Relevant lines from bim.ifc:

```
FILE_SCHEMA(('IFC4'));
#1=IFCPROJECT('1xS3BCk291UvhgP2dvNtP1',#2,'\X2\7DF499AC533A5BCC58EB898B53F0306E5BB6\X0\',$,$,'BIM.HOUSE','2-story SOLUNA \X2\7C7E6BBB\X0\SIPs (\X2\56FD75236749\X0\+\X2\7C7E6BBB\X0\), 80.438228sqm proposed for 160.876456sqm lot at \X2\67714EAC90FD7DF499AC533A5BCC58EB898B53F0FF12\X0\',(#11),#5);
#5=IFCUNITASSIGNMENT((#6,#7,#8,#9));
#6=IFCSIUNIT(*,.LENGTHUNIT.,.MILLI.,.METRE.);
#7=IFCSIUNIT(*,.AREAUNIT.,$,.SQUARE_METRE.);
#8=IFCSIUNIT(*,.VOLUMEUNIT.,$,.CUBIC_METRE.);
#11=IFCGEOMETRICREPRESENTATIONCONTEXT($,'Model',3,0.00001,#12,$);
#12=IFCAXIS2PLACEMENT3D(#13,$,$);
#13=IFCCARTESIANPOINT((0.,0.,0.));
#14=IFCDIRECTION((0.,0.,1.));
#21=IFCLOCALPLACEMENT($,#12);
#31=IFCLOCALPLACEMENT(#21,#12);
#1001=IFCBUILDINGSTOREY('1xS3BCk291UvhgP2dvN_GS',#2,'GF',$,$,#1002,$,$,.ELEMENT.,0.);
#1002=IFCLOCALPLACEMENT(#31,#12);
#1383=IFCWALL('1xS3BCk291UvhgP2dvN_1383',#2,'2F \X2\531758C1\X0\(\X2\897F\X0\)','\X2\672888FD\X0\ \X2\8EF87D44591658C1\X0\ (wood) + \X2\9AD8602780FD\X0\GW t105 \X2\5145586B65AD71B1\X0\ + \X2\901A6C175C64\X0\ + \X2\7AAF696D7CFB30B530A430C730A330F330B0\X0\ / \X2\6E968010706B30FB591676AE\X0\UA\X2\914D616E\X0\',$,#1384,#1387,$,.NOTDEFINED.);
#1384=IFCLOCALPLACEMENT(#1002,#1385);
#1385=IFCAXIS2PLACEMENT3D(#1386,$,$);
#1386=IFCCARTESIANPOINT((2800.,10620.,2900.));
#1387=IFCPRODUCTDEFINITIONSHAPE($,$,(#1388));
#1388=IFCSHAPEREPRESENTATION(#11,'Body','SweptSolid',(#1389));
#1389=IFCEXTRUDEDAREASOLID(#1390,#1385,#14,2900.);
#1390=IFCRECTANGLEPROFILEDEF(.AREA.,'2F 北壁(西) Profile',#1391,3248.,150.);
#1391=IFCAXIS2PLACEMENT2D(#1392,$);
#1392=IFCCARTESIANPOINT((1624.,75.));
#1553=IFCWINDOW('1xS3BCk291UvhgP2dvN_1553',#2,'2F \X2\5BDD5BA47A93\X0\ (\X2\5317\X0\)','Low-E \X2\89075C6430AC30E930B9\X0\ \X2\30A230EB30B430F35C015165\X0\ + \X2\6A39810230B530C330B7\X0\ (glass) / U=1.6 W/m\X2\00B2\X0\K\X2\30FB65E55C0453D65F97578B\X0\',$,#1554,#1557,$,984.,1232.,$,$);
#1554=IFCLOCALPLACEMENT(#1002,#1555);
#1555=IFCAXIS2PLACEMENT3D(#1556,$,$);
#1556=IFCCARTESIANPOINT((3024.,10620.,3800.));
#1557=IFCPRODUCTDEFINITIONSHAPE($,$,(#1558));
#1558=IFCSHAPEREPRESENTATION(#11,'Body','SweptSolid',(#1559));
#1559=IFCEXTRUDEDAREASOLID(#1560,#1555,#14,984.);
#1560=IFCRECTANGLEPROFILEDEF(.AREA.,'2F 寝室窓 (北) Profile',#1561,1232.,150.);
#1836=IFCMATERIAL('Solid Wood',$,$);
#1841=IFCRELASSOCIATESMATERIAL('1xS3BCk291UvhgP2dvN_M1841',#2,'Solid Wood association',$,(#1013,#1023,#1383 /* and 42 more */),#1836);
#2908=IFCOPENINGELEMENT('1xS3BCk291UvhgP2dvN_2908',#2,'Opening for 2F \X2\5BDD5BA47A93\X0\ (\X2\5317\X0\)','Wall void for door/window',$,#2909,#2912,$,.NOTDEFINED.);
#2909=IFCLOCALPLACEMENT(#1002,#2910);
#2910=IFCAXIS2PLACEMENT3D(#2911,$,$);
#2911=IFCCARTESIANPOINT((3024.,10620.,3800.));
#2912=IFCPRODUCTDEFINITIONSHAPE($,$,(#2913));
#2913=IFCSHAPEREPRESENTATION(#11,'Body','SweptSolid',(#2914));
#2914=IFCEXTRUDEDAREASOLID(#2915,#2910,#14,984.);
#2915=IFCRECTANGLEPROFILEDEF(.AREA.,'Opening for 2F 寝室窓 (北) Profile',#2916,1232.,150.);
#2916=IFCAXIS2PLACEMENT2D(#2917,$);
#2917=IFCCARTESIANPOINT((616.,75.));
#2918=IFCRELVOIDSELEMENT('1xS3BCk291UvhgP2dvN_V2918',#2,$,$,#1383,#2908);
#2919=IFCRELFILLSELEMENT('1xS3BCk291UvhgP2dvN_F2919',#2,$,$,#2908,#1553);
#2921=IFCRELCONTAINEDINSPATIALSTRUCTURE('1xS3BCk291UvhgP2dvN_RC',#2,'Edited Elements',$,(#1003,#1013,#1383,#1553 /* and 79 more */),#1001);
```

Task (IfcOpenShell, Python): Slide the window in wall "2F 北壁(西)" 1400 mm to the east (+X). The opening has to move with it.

```python
import ifcopenshell
import ifcopenshell.api.geometry
import ifcopenshell.util.placement

model = ifcopenshell.open("bim.ifc")

window = model.by_id(1553)
opening = window.FillsVoids[0].RelatingOpeningElement
wall = opening.VoidsElements[0].RelatingBuildingElement

wall_matrix = ifcopenshell.util.placement.get_local_placement(wall.ObjectPlacement)
shift = wall_matrix[:3, 0] * 1400.0
before = ifcopenshell.util.placement.get_local_placement(window.ObjectPlacement)[:3, 3].copy()

# The window is not placed relative to its opening, so move both.
for product in (opening, window):
    matrix = ifcopenshell.util.placement.get_local_placement(product.ObjectPlacement)
    matrix[:3, 3] += shift
    ifcopenshell.api.geometry.edit_object_placement(model, product=product, matrix=matrix, is_si=False)

after = ifcopenshell.util.placement.get_local_placement(window.ObjectPlacement)[:3, 3]
print("window moved by", (after - before).round(3) + 0.0)

model.write("bim_updated.ifc")
```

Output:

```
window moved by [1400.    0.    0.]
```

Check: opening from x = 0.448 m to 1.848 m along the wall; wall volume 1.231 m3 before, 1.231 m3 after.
